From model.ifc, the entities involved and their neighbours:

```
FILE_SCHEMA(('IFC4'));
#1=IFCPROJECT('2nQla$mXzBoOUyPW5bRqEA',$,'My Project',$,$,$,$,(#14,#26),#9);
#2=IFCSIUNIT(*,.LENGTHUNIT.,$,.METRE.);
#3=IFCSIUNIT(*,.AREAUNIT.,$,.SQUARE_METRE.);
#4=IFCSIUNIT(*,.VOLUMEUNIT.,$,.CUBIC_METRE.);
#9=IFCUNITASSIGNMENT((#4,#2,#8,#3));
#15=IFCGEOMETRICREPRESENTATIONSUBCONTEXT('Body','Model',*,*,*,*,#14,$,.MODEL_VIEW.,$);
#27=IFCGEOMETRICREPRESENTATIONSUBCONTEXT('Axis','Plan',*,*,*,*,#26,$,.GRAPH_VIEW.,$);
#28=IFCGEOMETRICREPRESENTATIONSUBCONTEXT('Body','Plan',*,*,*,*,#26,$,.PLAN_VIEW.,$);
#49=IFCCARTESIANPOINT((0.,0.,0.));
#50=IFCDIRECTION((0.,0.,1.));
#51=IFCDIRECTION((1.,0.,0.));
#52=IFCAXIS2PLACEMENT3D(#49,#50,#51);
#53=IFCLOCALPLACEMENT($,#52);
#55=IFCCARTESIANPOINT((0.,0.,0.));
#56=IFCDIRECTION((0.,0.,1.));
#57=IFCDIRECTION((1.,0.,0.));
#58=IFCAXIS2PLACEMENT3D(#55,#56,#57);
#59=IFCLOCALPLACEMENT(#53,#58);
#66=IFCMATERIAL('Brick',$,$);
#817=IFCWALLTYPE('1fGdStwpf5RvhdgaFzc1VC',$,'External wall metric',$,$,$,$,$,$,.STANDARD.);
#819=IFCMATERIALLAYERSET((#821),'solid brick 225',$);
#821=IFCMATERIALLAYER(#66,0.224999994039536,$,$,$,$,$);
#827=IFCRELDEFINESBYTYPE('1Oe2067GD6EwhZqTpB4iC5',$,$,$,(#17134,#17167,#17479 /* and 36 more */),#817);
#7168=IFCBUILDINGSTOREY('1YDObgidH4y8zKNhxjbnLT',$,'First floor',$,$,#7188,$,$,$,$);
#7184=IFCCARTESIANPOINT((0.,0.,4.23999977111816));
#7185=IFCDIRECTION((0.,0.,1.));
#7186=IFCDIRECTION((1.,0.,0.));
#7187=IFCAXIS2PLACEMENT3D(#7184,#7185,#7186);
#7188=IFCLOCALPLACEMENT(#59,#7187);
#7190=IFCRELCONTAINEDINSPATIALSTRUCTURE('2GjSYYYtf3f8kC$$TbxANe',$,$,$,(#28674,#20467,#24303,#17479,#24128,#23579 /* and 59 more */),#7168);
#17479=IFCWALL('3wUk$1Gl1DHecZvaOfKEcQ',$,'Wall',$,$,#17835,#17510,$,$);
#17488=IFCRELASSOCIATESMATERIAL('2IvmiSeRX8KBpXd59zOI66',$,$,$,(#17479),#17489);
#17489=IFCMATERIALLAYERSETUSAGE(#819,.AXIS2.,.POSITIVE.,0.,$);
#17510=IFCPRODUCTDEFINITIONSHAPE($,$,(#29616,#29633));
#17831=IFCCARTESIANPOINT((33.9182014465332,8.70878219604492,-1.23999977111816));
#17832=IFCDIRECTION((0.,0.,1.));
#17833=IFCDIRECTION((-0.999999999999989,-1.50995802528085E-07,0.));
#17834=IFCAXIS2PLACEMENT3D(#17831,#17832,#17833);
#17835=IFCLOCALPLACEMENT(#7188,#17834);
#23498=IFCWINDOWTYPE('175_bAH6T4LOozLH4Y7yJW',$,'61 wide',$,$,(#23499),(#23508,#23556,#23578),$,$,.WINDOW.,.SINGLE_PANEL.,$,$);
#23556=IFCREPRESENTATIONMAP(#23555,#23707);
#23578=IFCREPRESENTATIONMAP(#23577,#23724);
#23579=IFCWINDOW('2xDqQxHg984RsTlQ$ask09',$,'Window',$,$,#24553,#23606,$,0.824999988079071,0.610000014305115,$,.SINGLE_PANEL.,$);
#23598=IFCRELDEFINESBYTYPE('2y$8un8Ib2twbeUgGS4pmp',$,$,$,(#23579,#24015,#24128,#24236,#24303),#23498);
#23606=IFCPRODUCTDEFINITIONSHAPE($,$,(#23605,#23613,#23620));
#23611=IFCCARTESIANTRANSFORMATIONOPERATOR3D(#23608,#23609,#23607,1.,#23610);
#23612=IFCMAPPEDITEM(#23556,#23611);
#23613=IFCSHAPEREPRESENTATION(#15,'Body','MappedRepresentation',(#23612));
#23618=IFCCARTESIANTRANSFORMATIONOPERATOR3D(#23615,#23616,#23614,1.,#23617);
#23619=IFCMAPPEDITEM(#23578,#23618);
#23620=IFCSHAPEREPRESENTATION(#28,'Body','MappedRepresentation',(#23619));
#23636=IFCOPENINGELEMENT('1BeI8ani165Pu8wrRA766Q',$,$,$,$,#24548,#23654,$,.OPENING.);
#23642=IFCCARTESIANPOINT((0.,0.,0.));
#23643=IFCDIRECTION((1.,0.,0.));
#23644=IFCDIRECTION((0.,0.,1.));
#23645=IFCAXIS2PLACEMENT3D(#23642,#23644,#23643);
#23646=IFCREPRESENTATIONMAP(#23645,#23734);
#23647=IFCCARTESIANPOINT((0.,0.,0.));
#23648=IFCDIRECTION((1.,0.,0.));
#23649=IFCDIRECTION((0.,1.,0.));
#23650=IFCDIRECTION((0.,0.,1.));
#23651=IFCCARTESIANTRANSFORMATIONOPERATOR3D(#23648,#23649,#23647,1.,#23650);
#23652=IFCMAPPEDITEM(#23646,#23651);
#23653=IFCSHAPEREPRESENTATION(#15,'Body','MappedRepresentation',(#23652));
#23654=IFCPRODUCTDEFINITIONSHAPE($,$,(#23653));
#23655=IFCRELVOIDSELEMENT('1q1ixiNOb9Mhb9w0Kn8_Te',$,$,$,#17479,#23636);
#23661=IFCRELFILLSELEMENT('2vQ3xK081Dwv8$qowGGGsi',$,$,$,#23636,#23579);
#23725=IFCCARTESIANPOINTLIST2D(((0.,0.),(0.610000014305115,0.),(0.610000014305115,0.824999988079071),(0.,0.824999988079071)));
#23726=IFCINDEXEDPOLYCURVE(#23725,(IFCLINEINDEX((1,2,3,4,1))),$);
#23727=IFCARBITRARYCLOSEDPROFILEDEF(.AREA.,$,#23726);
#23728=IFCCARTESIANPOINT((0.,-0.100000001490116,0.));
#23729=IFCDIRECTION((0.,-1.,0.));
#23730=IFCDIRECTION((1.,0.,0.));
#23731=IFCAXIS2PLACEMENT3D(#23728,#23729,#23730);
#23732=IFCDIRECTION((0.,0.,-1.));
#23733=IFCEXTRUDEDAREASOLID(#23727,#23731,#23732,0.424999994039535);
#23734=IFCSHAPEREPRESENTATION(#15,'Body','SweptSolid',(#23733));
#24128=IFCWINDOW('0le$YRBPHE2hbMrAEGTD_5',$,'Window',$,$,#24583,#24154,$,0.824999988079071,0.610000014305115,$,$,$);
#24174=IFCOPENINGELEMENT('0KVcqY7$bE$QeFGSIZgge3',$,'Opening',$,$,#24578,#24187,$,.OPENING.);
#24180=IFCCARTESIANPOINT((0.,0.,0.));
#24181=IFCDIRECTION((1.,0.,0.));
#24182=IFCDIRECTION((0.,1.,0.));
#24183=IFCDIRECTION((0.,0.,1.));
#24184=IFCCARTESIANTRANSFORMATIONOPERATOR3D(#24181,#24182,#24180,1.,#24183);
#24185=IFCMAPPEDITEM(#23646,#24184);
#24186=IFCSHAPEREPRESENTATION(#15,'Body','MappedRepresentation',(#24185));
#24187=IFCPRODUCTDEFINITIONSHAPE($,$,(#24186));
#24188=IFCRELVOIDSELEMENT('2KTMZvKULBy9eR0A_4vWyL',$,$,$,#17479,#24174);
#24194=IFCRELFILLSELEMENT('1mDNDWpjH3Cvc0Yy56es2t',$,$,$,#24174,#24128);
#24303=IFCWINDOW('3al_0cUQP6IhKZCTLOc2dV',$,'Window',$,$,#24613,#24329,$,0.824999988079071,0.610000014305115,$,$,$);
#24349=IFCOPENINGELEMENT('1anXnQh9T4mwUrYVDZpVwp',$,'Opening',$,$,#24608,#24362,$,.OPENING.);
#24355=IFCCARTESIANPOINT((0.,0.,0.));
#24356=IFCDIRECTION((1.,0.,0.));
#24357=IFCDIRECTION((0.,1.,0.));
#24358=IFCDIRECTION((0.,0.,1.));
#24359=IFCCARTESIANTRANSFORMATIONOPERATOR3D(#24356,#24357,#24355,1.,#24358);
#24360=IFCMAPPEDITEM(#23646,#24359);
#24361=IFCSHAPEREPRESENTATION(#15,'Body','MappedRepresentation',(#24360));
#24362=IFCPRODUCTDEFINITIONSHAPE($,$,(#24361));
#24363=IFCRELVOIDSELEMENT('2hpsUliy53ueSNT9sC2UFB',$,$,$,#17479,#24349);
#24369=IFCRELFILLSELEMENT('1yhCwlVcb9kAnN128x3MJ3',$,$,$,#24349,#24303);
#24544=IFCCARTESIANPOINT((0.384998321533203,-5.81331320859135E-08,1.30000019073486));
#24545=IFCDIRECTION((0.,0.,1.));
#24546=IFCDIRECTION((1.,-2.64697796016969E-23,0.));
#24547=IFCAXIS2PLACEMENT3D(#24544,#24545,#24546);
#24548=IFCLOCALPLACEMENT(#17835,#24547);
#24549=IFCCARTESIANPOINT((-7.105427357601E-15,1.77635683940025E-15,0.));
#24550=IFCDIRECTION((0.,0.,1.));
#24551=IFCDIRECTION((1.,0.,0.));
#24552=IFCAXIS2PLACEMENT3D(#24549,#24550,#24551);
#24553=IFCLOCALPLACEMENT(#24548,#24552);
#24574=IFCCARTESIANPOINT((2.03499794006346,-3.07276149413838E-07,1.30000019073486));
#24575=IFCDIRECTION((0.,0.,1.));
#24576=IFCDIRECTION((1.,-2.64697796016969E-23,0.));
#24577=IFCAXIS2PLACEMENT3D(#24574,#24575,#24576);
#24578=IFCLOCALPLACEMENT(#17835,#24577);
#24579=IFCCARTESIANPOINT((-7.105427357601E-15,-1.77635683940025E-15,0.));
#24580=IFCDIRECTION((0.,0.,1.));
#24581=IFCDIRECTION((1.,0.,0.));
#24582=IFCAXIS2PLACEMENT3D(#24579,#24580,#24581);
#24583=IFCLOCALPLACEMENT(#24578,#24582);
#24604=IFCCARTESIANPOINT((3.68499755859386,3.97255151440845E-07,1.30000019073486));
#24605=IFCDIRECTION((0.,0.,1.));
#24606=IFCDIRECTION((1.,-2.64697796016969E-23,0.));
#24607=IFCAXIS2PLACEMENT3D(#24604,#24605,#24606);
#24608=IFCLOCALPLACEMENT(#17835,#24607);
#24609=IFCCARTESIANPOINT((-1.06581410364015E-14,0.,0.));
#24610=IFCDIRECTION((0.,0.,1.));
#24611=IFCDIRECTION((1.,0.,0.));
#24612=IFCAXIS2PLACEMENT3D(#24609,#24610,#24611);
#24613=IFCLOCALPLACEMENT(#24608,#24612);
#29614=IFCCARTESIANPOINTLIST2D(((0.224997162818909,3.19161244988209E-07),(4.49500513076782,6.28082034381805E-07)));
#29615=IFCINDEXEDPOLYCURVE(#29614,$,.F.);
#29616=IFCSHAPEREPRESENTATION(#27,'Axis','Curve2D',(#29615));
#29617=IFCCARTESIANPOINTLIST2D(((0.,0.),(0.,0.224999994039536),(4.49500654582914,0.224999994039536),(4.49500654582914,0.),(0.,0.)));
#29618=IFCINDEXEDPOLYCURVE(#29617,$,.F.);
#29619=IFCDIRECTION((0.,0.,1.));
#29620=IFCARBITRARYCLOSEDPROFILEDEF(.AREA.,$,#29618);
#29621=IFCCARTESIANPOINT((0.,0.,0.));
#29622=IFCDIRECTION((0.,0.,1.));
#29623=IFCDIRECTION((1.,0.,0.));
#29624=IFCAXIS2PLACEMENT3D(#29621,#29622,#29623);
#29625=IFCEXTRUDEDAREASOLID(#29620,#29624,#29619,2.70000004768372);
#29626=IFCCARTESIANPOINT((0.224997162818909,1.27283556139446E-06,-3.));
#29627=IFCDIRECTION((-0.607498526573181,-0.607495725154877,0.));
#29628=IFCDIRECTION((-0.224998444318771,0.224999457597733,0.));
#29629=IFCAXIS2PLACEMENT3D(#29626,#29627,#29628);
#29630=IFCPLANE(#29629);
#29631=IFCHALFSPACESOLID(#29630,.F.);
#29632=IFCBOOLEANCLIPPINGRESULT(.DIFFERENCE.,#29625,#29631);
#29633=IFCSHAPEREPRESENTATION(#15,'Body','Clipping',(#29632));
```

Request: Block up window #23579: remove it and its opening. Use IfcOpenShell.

```python
import ifcopenshell
import ifcopenshell.api.feature
import ifcopenshell.api.root
import ifcopenshell.geom
import ifcopenshell.util.shape

model = ifcopenshell.open("model.ifc")
settings = ifcopenshell.geom.settings()


def volume(element):
    """Net volume in cubic metres, openings subtracted."""
    shape = ifcopenshell.geom.create_shape(settings, element)
    return ifcopenshell.util.shape.get_volume(shape.geometry)


window = model.by_guid("2xDqQxHg984RsTlQ$ask09")
opening = window.FillsVoids[0].RelatingOpeningElement
wall = opening.VoidsElements[0].RelatingBuildingElement
before = volume(wall)

ifcopenshell.api.root.remove_product(model, product=window)
ifcopenshell.api.feature.remove_feature(model, feature=opening)

after = volume(wall)

print(f"wall volume {before:.3f} -> {after:.3f} m3")

model.write("model_updated.ifc")
```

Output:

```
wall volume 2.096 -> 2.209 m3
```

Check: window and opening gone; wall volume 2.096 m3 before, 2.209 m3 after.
